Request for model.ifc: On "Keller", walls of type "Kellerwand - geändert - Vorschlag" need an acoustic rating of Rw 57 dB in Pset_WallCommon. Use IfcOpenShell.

First a look at what the model holds.

```python
import ifcopenshell
import ifcopenshell.util.element

model = ifcopenshell.open("model.ifc")
print(model.schema)
storey = next(s for s in model.by_type("IfcBuildingStorey") if s.Name == "Keller")
walls = [e for e in ifcopenshell.util.element.get_decomposition(storey) if e.is_a("IfcWall")]
seen = {}
for e in walls:
    element_type = ifcopenshell.util.element.get_type(e)
    key = (element_type.Name if element_type != e and element_type else None, ifcopenshell.util.element.get_pset(e, "Pset_WallCommon", "AcousticRating"))
    seen[key] = seen.get(key, 0) + 1
for (name, value), count in sorted(seen.items(), key=str):
    print(count, "x", name, "|", value)
```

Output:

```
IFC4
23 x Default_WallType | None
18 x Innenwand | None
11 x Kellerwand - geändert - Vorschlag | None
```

```python
import ifcopenshell
import ifcopenshell.api.pset
import ifcopenshell.util.element

model = ifcopenshell.open("model.ifc")

storey = next(s for s in model.by_type("IfcBuildingStorey") if s.Name == "Keller")
walls = [e for e in ifcopenshell.util.element.get_decomposition(storey) if e.is_a("IfcWall")]

count = 0
for e in walls:
    element_type = ifcopenshell.util.element.get_type(e)
    if element_type in (None, e) or element_type.Name != "Kellerwand - geändert - Vorschlag":
        continue
    # add_pset returns the element's existing set when there is one.
    pset = ifcopenshell.api.pset.add_pset(model, product=e, name="Pset_WallCommon")
    ifcopenshell.api.pset.edit_pset(model, pset=pset, properties={"AcousticRating": "Rw 57 dB"})
    count += 1

print(count, "walls updated")

model.write("model_v2.ifc")
```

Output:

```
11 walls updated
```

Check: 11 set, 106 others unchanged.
